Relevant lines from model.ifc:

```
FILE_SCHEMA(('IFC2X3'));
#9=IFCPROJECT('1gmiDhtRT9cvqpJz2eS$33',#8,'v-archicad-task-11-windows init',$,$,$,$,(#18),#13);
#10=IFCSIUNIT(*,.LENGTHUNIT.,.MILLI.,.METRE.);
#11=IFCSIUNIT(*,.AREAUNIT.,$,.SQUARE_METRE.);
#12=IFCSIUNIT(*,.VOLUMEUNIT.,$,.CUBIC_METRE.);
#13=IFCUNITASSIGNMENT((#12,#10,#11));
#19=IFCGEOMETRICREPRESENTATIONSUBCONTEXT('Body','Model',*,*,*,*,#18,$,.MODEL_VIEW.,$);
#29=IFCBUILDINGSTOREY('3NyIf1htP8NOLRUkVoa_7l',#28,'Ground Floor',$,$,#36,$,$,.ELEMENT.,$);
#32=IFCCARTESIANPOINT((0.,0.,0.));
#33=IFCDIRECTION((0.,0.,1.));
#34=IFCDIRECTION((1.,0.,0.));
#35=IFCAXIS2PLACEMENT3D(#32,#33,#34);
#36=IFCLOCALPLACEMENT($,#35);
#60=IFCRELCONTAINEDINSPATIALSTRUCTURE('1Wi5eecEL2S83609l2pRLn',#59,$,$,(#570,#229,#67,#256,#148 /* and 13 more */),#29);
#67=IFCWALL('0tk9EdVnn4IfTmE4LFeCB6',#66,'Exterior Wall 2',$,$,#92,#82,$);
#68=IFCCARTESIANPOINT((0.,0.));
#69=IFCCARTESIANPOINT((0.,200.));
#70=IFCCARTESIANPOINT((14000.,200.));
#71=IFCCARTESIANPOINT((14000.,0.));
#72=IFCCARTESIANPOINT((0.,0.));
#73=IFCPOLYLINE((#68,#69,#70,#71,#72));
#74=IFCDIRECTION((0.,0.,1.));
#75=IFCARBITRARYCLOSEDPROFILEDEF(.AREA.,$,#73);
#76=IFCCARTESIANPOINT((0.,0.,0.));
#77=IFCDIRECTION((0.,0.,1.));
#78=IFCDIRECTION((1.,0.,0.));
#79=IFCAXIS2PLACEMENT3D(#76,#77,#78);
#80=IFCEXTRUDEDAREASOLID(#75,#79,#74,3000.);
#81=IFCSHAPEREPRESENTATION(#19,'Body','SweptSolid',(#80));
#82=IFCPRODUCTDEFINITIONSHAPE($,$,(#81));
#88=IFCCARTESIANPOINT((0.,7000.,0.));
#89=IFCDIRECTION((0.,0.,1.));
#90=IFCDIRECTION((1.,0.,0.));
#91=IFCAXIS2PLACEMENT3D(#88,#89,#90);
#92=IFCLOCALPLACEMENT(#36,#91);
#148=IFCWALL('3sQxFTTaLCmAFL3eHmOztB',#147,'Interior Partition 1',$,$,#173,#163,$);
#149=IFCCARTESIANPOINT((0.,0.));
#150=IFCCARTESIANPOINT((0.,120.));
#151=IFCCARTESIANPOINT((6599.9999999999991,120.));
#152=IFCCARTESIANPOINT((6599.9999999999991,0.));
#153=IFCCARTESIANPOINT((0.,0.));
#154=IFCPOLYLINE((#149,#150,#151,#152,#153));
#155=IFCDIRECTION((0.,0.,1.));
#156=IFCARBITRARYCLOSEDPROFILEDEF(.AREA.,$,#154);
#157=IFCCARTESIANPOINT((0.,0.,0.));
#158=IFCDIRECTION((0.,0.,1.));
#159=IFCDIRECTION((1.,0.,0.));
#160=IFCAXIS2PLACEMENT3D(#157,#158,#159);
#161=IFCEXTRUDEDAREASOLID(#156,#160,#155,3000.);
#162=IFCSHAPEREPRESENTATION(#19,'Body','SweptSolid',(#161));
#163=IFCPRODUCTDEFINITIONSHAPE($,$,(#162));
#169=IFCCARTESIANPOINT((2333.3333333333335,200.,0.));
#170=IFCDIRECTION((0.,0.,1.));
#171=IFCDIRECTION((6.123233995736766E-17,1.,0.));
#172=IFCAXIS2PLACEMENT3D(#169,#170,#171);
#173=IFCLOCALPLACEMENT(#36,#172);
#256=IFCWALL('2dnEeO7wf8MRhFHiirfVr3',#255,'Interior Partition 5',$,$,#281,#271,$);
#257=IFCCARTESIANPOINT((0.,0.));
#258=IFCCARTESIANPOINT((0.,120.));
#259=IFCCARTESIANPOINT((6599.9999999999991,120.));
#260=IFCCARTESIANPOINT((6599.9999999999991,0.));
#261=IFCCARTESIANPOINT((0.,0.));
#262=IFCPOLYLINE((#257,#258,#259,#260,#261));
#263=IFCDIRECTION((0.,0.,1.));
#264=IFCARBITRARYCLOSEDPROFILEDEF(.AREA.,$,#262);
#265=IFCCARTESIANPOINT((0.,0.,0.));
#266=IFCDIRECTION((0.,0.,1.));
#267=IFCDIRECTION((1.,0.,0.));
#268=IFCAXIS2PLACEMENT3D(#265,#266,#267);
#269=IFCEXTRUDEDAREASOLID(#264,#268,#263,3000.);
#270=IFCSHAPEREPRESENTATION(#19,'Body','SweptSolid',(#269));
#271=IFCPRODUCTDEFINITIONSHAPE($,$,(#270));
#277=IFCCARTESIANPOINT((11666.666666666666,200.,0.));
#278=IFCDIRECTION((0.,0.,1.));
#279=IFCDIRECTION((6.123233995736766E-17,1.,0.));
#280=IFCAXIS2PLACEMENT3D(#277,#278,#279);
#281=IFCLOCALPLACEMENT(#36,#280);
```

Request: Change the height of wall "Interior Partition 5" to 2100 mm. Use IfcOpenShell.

```python
import ifcopenshell
import ifcopenshell.geom
import ifcopenshell.util.representation
import ifcopenshell.util.shape

model = ifcopenshell.open("model.ifc")
settings = ifcopenshell.geom.settings()


def volume(element):
    """Net volume in cubic metres, openings subtracted."""
    shape = ifcopenshell.geom.create_shape(settings, element)
    return ifcopenshell.util.shape.get_volume(shape.geometry)


wall = model.by_id(256)
before = volume(wall)

body = ifcopenshell.util.representation.get_representation(wall, "Model", "Body")
solid = body.Items[0]
old_height = solid.Depth
solid.Depth = 2100.0
after = volume(wall)

print(f"height {old_height:g} -> {solid.Depth:g}, volume {before:.3f} -> {after:.3f} m3")

model.write("model-out.ifc")
```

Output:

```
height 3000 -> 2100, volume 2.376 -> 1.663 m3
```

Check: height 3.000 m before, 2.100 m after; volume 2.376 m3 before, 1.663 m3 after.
